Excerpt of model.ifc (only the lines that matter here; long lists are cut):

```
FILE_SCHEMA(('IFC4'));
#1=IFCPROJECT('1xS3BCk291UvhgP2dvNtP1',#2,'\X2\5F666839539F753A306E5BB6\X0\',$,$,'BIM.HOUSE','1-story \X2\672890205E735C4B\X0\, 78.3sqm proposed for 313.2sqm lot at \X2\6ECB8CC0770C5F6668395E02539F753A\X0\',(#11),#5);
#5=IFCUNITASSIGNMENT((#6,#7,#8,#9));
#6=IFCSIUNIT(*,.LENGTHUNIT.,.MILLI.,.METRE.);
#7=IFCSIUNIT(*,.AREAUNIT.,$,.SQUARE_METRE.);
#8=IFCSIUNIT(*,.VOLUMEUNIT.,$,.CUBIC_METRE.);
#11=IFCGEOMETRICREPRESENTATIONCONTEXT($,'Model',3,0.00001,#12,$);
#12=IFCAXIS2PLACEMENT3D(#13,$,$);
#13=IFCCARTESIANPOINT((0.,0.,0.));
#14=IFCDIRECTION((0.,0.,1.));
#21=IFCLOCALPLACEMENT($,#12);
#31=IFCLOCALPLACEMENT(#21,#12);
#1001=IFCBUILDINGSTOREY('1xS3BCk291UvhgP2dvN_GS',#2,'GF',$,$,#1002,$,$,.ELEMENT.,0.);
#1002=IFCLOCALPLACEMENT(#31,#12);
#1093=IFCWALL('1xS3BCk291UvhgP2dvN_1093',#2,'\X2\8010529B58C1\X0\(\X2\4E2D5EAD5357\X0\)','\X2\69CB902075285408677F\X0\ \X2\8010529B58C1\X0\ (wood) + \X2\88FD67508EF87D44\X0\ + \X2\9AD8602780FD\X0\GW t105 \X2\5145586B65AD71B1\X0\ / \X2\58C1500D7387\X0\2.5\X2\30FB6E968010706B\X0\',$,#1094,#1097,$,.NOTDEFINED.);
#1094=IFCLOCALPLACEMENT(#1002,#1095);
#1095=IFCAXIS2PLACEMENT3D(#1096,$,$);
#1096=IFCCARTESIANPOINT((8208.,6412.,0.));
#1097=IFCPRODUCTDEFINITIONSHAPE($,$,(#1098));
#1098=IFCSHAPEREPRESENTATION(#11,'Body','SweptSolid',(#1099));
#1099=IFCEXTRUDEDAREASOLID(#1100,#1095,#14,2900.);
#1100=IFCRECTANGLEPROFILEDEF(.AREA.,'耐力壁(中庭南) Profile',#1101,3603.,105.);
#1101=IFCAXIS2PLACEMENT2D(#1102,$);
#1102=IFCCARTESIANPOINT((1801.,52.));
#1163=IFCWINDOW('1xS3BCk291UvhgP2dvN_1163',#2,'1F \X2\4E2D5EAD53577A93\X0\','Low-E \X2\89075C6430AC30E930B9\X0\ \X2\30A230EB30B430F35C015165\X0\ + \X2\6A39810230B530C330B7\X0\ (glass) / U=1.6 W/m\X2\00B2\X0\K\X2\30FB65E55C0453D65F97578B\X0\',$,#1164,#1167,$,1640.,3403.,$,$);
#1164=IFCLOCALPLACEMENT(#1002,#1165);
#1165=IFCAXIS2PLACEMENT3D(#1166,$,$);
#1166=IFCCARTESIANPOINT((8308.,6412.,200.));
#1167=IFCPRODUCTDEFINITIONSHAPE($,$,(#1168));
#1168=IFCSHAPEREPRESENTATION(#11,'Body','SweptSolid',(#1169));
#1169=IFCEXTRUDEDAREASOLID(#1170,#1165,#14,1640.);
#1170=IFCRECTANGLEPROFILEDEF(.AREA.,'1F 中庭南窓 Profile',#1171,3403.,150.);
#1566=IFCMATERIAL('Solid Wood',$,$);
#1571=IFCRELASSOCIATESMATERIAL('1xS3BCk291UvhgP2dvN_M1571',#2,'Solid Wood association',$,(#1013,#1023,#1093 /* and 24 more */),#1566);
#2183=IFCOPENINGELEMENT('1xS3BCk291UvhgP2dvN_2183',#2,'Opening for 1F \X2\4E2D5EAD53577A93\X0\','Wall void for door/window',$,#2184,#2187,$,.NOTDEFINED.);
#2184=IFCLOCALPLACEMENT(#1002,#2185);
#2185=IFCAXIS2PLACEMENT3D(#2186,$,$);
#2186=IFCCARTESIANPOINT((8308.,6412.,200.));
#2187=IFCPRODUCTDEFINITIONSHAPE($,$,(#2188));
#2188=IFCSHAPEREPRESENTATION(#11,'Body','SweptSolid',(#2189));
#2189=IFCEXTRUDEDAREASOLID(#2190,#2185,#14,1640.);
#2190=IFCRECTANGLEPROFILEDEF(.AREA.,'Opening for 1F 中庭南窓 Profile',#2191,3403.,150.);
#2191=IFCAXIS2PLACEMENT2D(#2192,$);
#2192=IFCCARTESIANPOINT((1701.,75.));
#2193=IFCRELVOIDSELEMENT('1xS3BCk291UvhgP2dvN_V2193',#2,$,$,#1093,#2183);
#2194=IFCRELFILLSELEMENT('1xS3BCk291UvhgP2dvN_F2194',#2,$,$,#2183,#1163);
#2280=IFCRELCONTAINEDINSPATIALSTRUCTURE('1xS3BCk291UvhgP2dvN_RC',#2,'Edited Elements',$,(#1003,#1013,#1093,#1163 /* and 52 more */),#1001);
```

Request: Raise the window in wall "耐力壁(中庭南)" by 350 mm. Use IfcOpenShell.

```python
import numpy as np
import ifcopenshell
import ifcopenshell.api.geometry
import ifcopenshell.util.placement
import ifcopenshell.util.unit

model = ifcopenshell.open("model.ifc")
unit_scale = ifcopenshell.util.unit.calculate_unit_scale(model)

window = model.by_guid("1xS3BCk291UvhgP2dvN_1163")
opening = window.FillsVoids[0].RelatingOpeningElement
dz = 0.35 / unit_scale

shift = np.array([0.0, 0.0, dz])
# The window is not placed relative to its opening, so move both.
for product in (opening, window):
    matrix = ifcopenshell.util.placement.get_local_placement(product.ObjectPlacement)
    matrix[:3, 3] += shift
    ifcopenshell.api.geometry.edit_object_placement(model, product=product, matrix=matrix, is_si=False)

print(f"moved by {dz * unit_scale:+.3f} m")

model.write("model-out.ifc")
```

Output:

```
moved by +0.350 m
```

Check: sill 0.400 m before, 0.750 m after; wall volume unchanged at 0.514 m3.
